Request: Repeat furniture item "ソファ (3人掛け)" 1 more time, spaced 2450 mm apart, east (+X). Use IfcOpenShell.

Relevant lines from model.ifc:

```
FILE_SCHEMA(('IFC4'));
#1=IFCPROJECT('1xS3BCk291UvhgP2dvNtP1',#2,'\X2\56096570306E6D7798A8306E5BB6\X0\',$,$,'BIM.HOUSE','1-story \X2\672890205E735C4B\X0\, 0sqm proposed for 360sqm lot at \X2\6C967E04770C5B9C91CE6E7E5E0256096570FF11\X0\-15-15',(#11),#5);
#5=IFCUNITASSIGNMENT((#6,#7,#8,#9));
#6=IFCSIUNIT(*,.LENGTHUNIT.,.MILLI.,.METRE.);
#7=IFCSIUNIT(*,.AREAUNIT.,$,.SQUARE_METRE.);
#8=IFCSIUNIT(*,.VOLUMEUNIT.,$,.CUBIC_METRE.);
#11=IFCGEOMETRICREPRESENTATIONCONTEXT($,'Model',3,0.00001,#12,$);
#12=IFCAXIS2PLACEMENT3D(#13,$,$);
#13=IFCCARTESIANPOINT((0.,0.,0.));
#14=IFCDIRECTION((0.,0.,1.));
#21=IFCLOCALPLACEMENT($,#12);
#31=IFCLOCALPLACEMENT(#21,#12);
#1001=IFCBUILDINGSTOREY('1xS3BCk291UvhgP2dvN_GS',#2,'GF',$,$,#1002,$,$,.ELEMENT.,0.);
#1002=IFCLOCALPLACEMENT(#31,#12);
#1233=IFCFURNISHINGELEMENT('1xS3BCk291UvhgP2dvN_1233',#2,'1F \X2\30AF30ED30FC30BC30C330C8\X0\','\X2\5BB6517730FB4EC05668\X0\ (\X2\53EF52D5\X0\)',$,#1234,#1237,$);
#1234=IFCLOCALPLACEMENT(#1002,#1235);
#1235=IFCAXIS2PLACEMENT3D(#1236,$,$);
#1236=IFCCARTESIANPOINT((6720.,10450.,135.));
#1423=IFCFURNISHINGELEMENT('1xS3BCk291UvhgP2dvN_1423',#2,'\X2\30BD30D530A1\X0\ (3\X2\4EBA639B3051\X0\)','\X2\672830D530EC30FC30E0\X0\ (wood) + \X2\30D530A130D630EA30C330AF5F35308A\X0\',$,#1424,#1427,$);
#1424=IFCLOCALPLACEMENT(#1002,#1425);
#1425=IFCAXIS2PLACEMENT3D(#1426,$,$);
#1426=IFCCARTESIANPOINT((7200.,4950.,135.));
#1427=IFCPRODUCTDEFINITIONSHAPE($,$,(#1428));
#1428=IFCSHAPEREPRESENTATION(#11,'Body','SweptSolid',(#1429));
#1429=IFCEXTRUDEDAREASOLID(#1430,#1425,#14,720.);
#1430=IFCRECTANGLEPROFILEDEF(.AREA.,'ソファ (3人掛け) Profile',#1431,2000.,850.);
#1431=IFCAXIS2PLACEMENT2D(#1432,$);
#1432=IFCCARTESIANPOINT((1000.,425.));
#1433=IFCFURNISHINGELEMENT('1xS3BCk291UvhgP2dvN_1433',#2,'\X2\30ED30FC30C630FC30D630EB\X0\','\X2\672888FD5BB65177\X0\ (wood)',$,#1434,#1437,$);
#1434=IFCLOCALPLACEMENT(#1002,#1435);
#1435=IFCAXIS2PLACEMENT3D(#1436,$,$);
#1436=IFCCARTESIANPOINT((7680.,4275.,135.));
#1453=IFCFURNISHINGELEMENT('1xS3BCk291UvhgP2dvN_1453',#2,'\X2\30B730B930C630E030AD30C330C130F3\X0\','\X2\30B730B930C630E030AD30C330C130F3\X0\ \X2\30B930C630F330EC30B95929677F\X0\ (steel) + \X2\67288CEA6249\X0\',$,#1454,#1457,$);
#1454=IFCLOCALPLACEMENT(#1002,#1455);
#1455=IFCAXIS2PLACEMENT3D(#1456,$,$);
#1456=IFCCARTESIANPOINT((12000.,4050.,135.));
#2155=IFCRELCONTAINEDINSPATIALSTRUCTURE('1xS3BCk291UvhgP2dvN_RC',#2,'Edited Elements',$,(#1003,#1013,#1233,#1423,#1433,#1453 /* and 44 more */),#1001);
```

```python
import numpy as np
import ifcopenshell
import ifcopenshell.api.geometry
import ifcopenshell.api.root
import ifcopenshell.util.element
import ifcopenshell.util.placement
import ifcopenshell.util.unit

model = ifcopenshell.open("model.ifc")
unit_scale = ifcopenshell.util.unit.calculate_unit_scale(model)


def reuse_history(source, copy):
    """copy_class also copies each property set's owner history, people and application; keep the originals."""
    for rel in copy.IsDefinedBy:
        if rel.is_a("IfcRelDefinesByProperties") and (history := rel.RelatingPropertyDefinition.OwnerHistory):
            rel.RelatingPropertyDefinition.OwnerHistory = source.OwnerHistory
            ifcopenshell.util.element.remove_deep2(model, history)


source = model.by_guid("1xS3BCk291UvhgP2dvN_1423")
base = ifcopenshell.util.placement.get_local_placement(source.ObjectPlacement)
step = np.array([1.0, 0.0, 0.0]) * 2.45 / unit_scale

for i in range(1, 2):
    copy = ifcopenshell.api.root.copy_class(model, product=source)
    copy.Representation = ifcopenshell.util.element.copy_deep(
        model, source.Representation, exclude=["IfcGeometricRepresentationContext", "IfcRepresentationMap"]
    )
    reuse_history(source, copy)
    matrix = base.copy()
    matrix[:3, 3] += i * step
    print("added at", matrix[:3, 3].round(3) + 0.0)
    ifcopenshell.api.geometry.edit_object_placement(model, product=copy, matrix=matrix, is_si=False)

model.write("model_updated.ifc")
```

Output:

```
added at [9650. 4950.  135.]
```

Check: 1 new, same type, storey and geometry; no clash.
